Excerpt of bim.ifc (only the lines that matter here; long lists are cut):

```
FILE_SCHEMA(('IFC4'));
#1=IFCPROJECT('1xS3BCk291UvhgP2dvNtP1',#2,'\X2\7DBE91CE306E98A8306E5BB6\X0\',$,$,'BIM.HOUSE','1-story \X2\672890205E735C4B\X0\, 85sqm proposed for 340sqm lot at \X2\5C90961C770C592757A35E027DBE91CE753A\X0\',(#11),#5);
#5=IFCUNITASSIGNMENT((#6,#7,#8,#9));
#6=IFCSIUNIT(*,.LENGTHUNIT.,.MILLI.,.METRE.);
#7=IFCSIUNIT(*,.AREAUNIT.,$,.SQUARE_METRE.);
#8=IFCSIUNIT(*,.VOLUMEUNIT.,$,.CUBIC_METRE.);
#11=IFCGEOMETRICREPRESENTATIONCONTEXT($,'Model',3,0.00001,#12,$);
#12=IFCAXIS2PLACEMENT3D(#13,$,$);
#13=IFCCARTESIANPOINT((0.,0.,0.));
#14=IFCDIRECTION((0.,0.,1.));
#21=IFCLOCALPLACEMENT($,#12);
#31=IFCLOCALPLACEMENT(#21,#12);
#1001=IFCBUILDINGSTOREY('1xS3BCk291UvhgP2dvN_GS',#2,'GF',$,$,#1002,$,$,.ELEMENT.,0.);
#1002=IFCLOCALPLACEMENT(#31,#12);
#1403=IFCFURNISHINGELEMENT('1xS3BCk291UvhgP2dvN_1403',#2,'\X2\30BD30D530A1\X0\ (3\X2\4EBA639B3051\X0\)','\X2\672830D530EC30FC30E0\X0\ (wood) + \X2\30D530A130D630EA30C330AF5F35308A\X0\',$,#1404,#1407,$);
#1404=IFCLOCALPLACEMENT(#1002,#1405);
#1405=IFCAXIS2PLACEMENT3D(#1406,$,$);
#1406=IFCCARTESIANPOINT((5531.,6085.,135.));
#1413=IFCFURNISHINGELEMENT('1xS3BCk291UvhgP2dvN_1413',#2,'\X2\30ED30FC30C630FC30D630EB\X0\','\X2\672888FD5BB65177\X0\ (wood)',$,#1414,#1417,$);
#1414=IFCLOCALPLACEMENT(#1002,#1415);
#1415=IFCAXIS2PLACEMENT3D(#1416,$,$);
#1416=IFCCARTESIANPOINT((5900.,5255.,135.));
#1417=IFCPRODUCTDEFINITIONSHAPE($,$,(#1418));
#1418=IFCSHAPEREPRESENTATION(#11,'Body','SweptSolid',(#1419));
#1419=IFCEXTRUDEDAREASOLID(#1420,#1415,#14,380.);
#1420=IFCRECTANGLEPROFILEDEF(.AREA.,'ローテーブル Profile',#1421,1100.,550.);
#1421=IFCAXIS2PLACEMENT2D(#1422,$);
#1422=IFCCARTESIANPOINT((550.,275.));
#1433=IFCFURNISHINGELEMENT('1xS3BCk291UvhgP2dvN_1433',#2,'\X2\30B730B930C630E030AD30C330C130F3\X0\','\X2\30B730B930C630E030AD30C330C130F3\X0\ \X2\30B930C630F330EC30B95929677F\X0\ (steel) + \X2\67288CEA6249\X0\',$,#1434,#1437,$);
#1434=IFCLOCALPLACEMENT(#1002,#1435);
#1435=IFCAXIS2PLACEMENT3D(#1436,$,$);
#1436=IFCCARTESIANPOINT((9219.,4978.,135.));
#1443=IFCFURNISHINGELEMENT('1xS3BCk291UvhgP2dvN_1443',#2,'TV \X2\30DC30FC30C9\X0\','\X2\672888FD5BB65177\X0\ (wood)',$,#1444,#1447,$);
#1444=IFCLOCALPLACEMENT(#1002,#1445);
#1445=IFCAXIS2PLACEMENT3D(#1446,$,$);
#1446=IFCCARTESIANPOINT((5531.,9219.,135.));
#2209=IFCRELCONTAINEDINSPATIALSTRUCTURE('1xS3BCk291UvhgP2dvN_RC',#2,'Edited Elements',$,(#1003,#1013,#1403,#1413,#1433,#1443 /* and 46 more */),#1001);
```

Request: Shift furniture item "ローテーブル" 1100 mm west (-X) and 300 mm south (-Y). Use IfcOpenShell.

```python
import ifcopenshell
import ifcopenshell.api.geometry
import ifcopenshell.util.placement

model = ifcopenshell.open("bim.ifc")

item = model.by_guid("1xS3BCk291UvhgP2dvN_1413")
matrix = ifcopenshell.util.placement.get_local_placement(item.ObjectPlacement)
matrix[0, 3] -= 1100.0
matrix[1, 3] -= 300.0
ifcopenshell.api.geometry.edit_object_placement(model, product=item, matrix=matrix, is_si=False)

print(ifcopenshell.util.placement.get_local_placement(item.ObjectPlacement).round(3) + 0.0)

model.write("bim_updated.ifc")
```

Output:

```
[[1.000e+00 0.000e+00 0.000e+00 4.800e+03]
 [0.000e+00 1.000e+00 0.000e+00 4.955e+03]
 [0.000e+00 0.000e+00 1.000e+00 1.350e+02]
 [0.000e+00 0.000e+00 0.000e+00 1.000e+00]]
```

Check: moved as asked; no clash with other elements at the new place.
